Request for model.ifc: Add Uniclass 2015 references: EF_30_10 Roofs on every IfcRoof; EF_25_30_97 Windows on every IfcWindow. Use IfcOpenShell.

First a look at what the model holds.

```python
import ifcopenshell

model = ifcopenshell.open("model.ifc")
print(model.schema)
print("classifications:", [c.Name for c in model.by_type("IfcClassification")])
for ifc_class in ("IfcDoor", "IfcRoof", "IfcStair", "IfcWall", "IfcWindow"):
    print(ifc_class, len(model.by_type(ifc_class)))
```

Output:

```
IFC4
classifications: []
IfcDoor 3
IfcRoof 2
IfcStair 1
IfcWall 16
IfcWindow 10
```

```python
import ifcopenshell
import ifcopenshell.api.classification

model = ifcopenshell.open("model.ifc")

system = ifcopenshell.api.classification.add_classification(model, classification="Uniclass 2015")

codes = {
    "IfcRoof": ("EF_30_10", "Roofs"),
    "IfcWindow": ("EF_25_30_97", "Windows"),
}
for ifc_class, (code, name) in codes.items():
    products = model.by_type(ifc_class)
    ifcopenshell.api.classification.add_reference(
        model, products=products, classification=system, identification=code, name=name
    )
    print(code, len(products))

model.write("model_v2.ifc")
```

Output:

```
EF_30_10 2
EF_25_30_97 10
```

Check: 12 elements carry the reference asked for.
